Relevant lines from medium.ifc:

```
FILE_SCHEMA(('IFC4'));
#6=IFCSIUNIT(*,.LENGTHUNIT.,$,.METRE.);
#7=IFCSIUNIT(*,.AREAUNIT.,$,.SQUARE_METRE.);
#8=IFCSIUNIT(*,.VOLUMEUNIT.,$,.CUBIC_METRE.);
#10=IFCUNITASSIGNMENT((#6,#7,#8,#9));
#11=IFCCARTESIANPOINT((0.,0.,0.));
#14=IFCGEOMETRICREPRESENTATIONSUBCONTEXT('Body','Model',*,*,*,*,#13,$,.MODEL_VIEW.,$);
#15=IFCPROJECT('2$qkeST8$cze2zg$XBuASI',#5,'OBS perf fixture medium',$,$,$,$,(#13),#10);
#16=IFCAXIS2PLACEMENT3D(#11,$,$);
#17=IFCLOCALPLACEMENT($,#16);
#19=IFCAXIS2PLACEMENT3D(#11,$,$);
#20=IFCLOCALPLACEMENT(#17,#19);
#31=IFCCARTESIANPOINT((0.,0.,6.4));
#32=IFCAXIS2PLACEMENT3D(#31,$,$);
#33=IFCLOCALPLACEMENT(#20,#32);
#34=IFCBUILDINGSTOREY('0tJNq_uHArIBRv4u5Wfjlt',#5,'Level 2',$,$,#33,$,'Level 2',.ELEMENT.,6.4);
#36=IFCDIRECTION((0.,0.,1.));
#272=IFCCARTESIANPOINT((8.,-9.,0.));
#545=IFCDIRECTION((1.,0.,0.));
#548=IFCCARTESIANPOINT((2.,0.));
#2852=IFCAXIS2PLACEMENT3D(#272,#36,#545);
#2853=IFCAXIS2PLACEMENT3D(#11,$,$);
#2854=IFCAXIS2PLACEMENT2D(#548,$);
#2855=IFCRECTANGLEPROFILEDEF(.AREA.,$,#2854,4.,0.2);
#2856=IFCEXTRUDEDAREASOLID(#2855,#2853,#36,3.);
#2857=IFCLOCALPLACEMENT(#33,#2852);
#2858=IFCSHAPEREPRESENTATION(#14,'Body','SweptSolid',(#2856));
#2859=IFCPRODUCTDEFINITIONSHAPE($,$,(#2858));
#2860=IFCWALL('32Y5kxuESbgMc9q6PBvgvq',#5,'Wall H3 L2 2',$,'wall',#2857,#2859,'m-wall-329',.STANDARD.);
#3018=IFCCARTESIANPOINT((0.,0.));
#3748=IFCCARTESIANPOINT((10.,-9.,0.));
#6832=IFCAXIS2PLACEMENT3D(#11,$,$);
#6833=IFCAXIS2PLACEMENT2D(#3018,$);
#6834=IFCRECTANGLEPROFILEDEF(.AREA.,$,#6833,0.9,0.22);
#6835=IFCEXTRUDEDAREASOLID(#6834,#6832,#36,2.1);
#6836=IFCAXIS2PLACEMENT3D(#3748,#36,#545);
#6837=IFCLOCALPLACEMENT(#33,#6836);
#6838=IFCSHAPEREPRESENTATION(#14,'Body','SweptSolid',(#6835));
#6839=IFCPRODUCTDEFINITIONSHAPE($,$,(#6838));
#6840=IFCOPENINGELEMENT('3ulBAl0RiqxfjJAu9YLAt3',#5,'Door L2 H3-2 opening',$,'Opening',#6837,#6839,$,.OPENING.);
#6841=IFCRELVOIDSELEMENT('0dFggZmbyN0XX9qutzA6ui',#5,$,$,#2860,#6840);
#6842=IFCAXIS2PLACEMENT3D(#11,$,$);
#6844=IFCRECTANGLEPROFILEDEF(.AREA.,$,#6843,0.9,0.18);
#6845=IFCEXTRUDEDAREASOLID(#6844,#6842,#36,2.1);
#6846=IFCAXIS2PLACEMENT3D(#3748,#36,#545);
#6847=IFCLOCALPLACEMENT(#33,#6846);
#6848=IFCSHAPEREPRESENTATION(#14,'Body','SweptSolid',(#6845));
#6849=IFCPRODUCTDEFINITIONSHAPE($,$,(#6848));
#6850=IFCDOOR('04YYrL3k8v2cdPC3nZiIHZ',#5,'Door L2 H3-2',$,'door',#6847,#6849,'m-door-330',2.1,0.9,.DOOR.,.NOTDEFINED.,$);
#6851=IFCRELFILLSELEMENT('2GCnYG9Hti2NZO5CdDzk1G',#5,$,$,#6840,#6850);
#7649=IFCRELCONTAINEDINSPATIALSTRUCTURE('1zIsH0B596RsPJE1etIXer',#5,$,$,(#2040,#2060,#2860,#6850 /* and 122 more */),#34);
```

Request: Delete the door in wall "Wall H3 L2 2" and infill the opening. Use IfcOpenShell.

```python
import ifcopenshell
import ifcopenshell.api.feature
import ifcopenshell.api.root
import ifcopenshell.geom
import ifcopenshell.util.shape

model = ifcopenshell.open("medium.ifc")
settings = ifcopenshell.geom.settings()


def volume(element):
    """Net volume in cubic metres, openings subtracted."""
    shape = ifcopenshell.geom.create_shape(settings, element)
    return ifcopenshell.util.shape.get_volume(shape.geometry)


door = model.by_guid("04YYrL3k8v2cdPC3nZiIHZ")
opening = door.FillsVoids[0].RelatingOpeningElement
wall = opening.VoidsElements[0].RelatingBuildingElement
before = volume(wall)

ifcopenshell.api.root.remove_product(model, product=door)
ifcopenshell.api.feature.remove_feature(model, feature=opening)

after = volume(wall)

print(f"wall volume {before:.3f} -> {after:.3f} m3")

model.write("medium_updated.ifc")
```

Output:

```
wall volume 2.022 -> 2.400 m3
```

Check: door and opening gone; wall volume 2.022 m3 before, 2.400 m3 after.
